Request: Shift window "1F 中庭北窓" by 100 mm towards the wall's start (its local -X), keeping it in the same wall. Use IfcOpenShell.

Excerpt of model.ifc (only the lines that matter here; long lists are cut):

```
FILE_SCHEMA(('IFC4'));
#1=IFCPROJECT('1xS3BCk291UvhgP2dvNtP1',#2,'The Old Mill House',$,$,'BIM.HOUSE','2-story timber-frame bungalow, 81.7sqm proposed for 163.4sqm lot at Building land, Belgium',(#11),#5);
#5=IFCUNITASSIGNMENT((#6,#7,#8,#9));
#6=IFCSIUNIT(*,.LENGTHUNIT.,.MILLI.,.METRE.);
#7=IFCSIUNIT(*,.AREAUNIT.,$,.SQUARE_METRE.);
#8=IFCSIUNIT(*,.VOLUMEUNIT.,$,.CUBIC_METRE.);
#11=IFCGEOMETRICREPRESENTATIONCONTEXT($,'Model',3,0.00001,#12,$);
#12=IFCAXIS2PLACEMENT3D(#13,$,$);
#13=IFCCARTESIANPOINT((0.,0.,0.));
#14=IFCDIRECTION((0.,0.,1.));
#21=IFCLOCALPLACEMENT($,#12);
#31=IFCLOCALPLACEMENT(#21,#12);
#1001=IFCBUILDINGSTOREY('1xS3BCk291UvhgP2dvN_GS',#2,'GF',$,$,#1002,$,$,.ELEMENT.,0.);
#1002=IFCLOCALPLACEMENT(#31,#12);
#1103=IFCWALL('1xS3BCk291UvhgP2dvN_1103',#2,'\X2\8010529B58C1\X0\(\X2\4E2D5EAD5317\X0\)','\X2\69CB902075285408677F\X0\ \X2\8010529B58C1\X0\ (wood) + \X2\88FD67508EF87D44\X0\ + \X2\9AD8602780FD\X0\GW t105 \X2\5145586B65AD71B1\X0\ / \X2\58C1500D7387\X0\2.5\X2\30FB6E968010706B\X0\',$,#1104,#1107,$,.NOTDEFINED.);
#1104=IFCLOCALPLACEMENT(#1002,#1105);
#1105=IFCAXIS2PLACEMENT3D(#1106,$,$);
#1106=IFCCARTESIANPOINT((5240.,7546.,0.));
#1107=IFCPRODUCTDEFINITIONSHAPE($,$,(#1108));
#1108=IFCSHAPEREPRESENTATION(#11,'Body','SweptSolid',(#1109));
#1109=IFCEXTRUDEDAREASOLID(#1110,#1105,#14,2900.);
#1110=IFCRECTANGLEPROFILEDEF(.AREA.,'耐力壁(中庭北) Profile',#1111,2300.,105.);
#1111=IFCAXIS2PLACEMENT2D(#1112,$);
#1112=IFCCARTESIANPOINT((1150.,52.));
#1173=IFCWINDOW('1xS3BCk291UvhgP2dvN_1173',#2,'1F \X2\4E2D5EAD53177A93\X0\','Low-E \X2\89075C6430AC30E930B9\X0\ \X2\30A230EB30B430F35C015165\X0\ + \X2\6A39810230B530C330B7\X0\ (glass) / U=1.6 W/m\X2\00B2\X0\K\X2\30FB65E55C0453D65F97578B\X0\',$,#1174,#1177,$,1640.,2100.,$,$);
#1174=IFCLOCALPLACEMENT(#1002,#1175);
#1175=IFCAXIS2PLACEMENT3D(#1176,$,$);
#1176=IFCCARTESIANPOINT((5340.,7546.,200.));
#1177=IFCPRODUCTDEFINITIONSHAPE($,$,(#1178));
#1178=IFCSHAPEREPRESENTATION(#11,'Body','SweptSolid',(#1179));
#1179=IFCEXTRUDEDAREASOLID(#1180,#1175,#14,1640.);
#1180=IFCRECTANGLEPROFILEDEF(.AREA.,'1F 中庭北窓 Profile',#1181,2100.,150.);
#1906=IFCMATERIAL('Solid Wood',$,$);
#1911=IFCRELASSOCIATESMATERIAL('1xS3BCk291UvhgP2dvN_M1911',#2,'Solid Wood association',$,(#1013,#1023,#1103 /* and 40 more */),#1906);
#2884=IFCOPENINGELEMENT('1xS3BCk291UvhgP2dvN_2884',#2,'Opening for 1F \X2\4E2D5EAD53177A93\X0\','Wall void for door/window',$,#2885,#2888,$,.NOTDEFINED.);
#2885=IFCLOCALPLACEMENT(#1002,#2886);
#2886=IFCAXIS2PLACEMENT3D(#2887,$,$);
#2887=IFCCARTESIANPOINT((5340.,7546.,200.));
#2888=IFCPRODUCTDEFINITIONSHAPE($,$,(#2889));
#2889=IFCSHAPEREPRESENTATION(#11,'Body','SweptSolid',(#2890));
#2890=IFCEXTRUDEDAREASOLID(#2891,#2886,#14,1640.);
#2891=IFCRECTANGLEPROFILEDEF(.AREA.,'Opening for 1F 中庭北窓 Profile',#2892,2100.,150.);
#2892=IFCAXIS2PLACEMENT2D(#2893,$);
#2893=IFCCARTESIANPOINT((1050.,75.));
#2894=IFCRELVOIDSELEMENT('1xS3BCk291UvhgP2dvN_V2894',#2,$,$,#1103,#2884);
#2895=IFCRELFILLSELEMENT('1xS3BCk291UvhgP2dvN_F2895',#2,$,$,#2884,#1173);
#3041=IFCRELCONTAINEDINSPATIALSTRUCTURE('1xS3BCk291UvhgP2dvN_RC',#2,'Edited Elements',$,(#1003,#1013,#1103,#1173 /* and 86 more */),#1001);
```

```python
import ifcopenshell
import ifcopenshell.api.geometry
import ifcopenshell.util.placement
import ifcopenshell.util.unit

model = ifcopenshell.open("model.ifc")
unit_scale = ifcopenshell.util.unit.calculate_unit_scale(model)

window = model.by_id(1173)
opening = window.FillsVoids[0].RelatingOpeningElement
wall = opening.VoidsElements[0].RelatingBuildingElement

wall_matrix = ifcopenshell.util.placement.get_local_placement(wall.ObjectPlacement)
shift = wall_matrix[:3, 0] * -0.1 / unit_scale
before = ifcopenshell.util.placement.get_local_placement(window.ObjectPlacement)[:3, 3].copy()

# The window is not placed relative to its opening, so move both.
for product in (opening, window):
    matrix = ifcopenshell.util.placement.get_local_placement(product.ObjectPlacement)
    matrix[:3, 3] += shift
    ifcopenshell.api.geometry.edit_object_placement(model, product=product, matrix=matrix, is_si=False)

after = ifcopenshell.util.placement.get_local_placement(window.ObjectPlacement)[:3, 3]
print("window moved by", (after - before).round(3) + 0.0)

model.write("model_edited.ifc")
```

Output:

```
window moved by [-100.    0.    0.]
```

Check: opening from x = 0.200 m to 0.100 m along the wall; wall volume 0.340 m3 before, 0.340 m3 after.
